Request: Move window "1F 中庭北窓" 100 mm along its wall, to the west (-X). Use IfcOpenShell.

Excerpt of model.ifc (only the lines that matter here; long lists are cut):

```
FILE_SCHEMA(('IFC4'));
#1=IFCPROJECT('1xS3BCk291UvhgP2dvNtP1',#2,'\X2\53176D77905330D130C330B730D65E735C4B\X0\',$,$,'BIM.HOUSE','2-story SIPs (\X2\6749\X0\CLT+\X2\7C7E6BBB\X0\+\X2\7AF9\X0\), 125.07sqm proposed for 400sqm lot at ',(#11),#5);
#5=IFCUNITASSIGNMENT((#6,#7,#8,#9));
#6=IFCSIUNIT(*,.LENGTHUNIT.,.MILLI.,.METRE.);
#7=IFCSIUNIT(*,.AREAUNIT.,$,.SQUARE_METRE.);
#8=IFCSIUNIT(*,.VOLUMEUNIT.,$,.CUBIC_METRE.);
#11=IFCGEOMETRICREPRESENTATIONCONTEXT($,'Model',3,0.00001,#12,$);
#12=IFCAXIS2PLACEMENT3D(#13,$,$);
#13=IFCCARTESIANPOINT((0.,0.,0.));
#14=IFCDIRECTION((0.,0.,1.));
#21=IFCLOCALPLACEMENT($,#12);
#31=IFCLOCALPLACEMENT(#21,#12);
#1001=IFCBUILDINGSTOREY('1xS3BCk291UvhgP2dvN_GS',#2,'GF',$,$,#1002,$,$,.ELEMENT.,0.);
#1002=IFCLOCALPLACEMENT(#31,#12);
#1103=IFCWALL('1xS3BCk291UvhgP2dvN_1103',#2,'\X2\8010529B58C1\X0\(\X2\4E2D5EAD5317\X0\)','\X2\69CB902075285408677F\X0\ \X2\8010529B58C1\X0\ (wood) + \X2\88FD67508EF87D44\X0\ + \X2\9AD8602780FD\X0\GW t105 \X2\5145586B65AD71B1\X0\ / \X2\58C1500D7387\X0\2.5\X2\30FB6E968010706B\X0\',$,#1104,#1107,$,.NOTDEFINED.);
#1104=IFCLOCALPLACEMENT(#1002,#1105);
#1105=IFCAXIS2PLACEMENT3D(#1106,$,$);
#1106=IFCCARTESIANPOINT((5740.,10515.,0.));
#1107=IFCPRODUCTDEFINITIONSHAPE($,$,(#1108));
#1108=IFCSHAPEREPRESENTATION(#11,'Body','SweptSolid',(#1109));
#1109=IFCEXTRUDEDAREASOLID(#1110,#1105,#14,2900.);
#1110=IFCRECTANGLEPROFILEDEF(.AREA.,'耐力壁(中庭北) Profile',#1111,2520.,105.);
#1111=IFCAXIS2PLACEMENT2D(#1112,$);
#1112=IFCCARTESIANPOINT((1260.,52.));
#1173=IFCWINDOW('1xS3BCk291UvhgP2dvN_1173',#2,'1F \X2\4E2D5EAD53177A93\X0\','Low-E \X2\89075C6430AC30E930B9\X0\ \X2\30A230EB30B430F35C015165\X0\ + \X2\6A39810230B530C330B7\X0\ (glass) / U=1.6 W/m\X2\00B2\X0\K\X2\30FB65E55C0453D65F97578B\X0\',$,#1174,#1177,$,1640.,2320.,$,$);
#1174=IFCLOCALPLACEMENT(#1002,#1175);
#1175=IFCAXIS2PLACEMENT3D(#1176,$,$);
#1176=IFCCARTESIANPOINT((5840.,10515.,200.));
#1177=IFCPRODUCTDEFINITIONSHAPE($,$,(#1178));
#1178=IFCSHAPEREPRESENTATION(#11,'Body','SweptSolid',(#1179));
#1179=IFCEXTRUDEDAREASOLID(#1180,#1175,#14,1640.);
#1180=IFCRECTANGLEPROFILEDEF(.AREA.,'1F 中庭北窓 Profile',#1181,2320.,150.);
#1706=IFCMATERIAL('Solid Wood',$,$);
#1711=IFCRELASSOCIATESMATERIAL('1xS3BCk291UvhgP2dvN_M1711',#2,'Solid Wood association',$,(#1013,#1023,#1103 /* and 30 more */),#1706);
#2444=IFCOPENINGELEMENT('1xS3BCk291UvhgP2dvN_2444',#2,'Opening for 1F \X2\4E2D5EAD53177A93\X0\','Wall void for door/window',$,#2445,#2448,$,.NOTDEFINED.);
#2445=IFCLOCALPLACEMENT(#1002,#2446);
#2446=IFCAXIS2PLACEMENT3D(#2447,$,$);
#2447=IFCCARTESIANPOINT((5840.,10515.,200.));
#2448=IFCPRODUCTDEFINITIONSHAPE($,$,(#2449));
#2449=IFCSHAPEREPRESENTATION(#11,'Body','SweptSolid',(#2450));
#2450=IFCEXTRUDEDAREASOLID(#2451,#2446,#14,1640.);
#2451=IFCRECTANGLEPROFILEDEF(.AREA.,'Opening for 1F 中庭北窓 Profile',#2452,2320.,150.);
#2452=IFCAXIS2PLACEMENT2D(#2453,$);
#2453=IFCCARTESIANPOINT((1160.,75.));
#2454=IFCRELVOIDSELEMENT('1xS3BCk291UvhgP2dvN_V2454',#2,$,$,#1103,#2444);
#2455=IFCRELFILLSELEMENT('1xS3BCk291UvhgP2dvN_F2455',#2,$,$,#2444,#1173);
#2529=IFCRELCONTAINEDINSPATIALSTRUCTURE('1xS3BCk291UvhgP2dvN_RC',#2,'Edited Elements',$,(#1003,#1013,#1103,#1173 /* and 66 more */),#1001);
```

```python
import ifcopenshell
import ifcopenshell.api.geometry
import ifcopenshell.util.placement
import ifcopenshell.util.unit

model = ifcopenshell.open("model.ifc")
unit_scale = ifcopenshell.util.unit.calculate_unit_scale(model)

window = model.by_id(1173)
opening = window.FillsVoids[0].RelatingOpeningElement
wall = opening.VoidsElements[0].RelatingBuildingElement

wall_matrix = ifcopenshell.util.placement.get_local_placement(wall.ObjectPlacement)
shift = wall_matrix[:3, 0] * -0.1 / unit_scale
before = ifcopenshell.util.placement.get_local_placement(window.ObjectPlacement)[:3, 3].copy()

# The window is not placed relative to its opening, so move both.
for product in (opening, window):
    matrix = ifcopenshell.util.placement.get_local_placement(product.ObjectPlacement)
    matrix[:3, 3] += shift
    ifcopenshell.api.geometry.edit_object_placement(model, product=product, matrix=matrix, is_si=False)

after = ifcopenshell.util.placement.get_local_placement(window.ObjectPlacement)[:3, 3]
print("window moved by", (after - before).round(3) + 0.0)

model.write("model_rev.ifc")
```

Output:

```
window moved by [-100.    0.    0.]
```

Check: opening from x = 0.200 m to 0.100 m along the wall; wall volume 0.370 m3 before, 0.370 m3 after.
